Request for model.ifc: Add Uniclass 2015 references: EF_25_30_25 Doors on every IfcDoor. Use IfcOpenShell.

First a look at what the model holds.

```python
import ifcopenshell

model = ifcopenshell.open("model.ifc")
print(model.schema)
print("classifications:", [c.Name for c in model.by_type("IfcClassification")])
for ifc_class in ("IfcDoor", "IfcRoof", "IfcStair", "IfcWall", "IfcWindow"):
    print(ifc_class, len(model.by_type(ifc_class)))
```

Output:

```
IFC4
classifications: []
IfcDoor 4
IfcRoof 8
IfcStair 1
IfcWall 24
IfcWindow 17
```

```python
import ifcopenshell
import ifcopenshell.api.classification

model = ifcopenshell.open("model.ifc")

system = ifcopenshell.api.classification.add_classification(model, classification="Uniclass 2015")

codes = {
    "IfcDoor": ("EF_25_30_25", "Doors"),
}
for ifc_class, (code, name) in codes.items():
    products = model.by_type(ifc_class)
    ifcopenshell.api.classification.add_reference(
        model, products=products, classification=system, identification=code, name=name
    )
    print(code, len(products))

model.write("model_updated.ifc")
```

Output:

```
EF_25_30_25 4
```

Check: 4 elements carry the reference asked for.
